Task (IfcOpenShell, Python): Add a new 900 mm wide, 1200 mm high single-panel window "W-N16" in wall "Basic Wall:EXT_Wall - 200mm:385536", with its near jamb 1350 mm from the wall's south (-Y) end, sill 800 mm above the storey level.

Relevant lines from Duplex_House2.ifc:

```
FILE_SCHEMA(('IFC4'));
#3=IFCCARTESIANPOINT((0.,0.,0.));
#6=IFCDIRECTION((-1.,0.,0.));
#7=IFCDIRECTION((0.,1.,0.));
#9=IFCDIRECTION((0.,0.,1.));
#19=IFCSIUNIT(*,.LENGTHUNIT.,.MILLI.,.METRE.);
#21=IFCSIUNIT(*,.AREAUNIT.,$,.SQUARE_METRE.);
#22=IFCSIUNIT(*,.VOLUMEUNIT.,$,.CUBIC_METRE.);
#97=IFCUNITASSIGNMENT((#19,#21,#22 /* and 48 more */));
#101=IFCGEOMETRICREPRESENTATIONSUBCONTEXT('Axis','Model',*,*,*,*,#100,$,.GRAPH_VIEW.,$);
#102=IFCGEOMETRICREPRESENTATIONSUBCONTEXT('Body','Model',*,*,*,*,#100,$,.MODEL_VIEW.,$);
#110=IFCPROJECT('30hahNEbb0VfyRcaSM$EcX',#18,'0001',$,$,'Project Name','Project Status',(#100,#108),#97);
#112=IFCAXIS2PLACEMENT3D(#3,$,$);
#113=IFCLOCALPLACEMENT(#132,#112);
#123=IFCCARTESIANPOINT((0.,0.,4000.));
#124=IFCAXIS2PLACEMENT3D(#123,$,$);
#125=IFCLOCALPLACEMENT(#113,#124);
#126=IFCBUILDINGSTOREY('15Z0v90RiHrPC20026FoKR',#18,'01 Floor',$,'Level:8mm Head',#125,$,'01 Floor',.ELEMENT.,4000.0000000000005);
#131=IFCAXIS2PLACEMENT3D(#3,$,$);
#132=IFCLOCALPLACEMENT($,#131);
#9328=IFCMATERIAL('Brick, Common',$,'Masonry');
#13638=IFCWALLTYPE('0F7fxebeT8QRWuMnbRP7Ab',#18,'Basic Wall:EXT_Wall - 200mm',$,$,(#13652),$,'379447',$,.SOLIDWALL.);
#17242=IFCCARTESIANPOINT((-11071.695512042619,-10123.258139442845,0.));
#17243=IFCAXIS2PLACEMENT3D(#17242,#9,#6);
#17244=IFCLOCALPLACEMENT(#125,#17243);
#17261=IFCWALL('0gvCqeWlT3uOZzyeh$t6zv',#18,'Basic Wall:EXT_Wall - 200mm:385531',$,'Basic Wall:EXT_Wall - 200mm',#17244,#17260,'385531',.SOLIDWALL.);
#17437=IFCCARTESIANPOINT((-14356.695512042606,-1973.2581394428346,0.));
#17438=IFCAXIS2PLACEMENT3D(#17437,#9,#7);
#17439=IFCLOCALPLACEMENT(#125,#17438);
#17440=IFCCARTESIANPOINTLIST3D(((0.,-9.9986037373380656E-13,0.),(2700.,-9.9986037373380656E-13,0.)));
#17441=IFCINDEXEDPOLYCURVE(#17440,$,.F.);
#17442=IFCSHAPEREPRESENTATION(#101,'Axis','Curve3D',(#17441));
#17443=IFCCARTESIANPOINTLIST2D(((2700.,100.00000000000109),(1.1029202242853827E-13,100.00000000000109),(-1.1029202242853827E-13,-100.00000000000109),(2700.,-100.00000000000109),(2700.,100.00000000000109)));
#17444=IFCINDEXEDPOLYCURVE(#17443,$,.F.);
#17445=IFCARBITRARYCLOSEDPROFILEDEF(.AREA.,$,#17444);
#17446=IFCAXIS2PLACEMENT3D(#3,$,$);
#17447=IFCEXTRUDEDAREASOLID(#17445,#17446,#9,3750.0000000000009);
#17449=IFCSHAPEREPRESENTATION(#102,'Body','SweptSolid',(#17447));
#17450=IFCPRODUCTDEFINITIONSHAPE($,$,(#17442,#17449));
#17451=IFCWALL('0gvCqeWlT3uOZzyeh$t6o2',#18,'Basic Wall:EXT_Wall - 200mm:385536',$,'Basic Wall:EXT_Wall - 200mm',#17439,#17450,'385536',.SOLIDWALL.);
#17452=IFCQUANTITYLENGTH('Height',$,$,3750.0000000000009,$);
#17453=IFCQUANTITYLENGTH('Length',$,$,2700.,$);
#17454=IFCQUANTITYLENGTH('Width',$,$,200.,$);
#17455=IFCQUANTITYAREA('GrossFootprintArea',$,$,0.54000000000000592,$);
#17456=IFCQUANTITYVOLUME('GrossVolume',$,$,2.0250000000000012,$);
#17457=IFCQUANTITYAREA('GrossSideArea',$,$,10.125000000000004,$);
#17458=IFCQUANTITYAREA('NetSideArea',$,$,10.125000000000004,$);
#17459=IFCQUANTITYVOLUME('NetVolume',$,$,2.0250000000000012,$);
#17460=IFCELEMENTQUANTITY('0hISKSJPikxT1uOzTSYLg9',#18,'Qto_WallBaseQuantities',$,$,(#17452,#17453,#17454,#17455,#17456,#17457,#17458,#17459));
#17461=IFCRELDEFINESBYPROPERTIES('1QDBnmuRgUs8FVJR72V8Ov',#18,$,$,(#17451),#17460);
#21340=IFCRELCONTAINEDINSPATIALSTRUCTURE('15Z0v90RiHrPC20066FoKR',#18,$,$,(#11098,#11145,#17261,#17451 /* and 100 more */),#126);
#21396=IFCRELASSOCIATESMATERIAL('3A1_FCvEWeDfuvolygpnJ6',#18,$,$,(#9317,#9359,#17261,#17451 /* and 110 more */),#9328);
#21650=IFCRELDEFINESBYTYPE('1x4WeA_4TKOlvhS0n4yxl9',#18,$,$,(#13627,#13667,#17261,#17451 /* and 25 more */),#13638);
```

```python
import numpy as np
import ifcopenshell
import ifcopenshell.api.feature
import ifcopenshell.api.geometry
import ifcopenshell.api.pset
import ifcopenshell.api.root
import ifcopenshell.api.spatial
import ifcopenshell.geom
import ifcopenshell.util.element
import ifcopenshell.util.placement
import ifcopenshell.util.representation
import ifcopenshell.util.shape
import ifcopenshell.util.unit

model = ifcopenshell.open("Duplex_House2.ifc")
unit_scale = ifcopenshell.util.unit.calculate_unit_scale(model)
area_scale = ifcopenshell.util.unit.calculate_unit_scale(model, "AREAUNIT")
volume_scale = ifcopenshell.util.unit.calculate_unit_scale(model, "VOLUMEUNIT")
settings = ifcopenshell.geom.settings()


def volume(element):
    """Net volume in cubic metres, openings subtracted."""
    shape = ifcopenshell.geom.create_shape(settings, element)
    return ifcopenshell.util.shape.get_volume(shape.geometry)


wall = model.by_id(17451)
storey = ifcopenshell.util.element.get_container(wall, ifc_class="IfcBuildingStorey")
context = ifcopenshell.util.representation.get_context(model, "Model", "Body", "MODEL_VIEW")
before = volume(wall)

width, height, from_end, sill = 0.9, 1.2, 1.35, 0.8  # metres

# The wall runs along its own X axis, and the end named is its -X end.
wall_shape = ifcopenshell.geom.create_shape(settings, wall)
x, y, z = ifcopenshell.util.shape.get_vertices(wall_shape.geometry).T
start = x.min() + from_end
face, thickness = float(y.min()), float(y.max() - y.min())
wall_matrix = ifcopenshell.util.placement.get_local_placement(wall.ObjectPlacement)
level = ifcopenshell.util.placement.get_local_placement(storey.ObjectPlacement)[2, 3]


def in_wall(x, y):
    """Placement at x, y metres in the wall's axes, at sill height."""
    matrix = wall_matrix.copy()
    matrix[:, 3] = wall_matrix @ np.array([x / unit_scale, y / unit_scale, 0.0, 1.0])
    matrix[2, 3] = level + sill / unit_scale
    return matrix


# Opening: a box that overshoots both wall faces by 50 mm.
opening = ifcopenshell.api.root.create_entity(model, ifc_class="IfcOpeningElement", predefined_type="OPENING")
box = ifcopenshell.api.geometry.add_wall_representation(
    model, context=context, length=width, height=height, thickness=thickness + 0.1
)
ifcopenshell.api.geometry.assign_representation(model, product=opening, representation=box)
ifcopenshell.api.geometry.edit_object_placement(model, product=opening, matrix=in_wall(start, face - 0.05), is_si=False)
ifcopenshell.api.feature.add_feature(model, feature=opening, element=wall)

window = ifcopenshell.api.root.create_entity(model, ifc_class="IfcWindow", name="W-N16", predefined_type="WINDOW")
window.OverallWidth, window.OverallHeight = width / unit_scale, height / unit_scale
window.PartitioningType = "SINGLE_PANEL"
body = ifcopenshell.api.geometry.add_window_representation(
    model,
    context=context,
    overall_width=window.OverallWidth,
    overall_height=window.OverallHeight,
    partition_type="SINGLE_PANEL",
)
ifcopenshell.api.geometry.assign_representation(model, product=window, representation=body)
ifcopenshell.api.spatial.assign_container(model, products=[window], relating_structure=storey)
ifcopenshell.api.feature.add_filling(model, opening=opening, element=window)

# Centre the window in the wall's thickness.
ifcopenshell.api.geometry.edit_object_placement(model, product=window, matrix=in_wall(start, face), is_si=False)
window_shape = ifcopenshell.geom.create_shape(settings, window)
depth = ifcopenshell.util.shape.get_vertices(window_shape.geometry)[:, 1]
offset = face + thickness / 2 - (depth.min() + depth.max()) / 2
ifcopenshell.api.geometry.edit_object_placement(model, product=window, matrix=in_wall(start, offset), is_si=False)

after = volume(wall)

# Update the wall's stored quantities.
qto = model.by_id(ifcopenshell.util.element.get_pset(wall, "Qto_WallBaseQuantities", should_inherit=False)["id"])
ifcopenshell.api.pset.edit_qto(model, qto=qto, properties={
    "NetSideArea": after / thickness / area_scale,
    "NetVolume": after / volume_scale,
})

print(f"wall volume {before:.3f} -> {after:.3f} m3")

model.write("Duplex_House2_edited.ifc")
```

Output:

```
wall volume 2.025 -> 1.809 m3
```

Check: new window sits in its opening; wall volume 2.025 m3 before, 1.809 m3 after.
